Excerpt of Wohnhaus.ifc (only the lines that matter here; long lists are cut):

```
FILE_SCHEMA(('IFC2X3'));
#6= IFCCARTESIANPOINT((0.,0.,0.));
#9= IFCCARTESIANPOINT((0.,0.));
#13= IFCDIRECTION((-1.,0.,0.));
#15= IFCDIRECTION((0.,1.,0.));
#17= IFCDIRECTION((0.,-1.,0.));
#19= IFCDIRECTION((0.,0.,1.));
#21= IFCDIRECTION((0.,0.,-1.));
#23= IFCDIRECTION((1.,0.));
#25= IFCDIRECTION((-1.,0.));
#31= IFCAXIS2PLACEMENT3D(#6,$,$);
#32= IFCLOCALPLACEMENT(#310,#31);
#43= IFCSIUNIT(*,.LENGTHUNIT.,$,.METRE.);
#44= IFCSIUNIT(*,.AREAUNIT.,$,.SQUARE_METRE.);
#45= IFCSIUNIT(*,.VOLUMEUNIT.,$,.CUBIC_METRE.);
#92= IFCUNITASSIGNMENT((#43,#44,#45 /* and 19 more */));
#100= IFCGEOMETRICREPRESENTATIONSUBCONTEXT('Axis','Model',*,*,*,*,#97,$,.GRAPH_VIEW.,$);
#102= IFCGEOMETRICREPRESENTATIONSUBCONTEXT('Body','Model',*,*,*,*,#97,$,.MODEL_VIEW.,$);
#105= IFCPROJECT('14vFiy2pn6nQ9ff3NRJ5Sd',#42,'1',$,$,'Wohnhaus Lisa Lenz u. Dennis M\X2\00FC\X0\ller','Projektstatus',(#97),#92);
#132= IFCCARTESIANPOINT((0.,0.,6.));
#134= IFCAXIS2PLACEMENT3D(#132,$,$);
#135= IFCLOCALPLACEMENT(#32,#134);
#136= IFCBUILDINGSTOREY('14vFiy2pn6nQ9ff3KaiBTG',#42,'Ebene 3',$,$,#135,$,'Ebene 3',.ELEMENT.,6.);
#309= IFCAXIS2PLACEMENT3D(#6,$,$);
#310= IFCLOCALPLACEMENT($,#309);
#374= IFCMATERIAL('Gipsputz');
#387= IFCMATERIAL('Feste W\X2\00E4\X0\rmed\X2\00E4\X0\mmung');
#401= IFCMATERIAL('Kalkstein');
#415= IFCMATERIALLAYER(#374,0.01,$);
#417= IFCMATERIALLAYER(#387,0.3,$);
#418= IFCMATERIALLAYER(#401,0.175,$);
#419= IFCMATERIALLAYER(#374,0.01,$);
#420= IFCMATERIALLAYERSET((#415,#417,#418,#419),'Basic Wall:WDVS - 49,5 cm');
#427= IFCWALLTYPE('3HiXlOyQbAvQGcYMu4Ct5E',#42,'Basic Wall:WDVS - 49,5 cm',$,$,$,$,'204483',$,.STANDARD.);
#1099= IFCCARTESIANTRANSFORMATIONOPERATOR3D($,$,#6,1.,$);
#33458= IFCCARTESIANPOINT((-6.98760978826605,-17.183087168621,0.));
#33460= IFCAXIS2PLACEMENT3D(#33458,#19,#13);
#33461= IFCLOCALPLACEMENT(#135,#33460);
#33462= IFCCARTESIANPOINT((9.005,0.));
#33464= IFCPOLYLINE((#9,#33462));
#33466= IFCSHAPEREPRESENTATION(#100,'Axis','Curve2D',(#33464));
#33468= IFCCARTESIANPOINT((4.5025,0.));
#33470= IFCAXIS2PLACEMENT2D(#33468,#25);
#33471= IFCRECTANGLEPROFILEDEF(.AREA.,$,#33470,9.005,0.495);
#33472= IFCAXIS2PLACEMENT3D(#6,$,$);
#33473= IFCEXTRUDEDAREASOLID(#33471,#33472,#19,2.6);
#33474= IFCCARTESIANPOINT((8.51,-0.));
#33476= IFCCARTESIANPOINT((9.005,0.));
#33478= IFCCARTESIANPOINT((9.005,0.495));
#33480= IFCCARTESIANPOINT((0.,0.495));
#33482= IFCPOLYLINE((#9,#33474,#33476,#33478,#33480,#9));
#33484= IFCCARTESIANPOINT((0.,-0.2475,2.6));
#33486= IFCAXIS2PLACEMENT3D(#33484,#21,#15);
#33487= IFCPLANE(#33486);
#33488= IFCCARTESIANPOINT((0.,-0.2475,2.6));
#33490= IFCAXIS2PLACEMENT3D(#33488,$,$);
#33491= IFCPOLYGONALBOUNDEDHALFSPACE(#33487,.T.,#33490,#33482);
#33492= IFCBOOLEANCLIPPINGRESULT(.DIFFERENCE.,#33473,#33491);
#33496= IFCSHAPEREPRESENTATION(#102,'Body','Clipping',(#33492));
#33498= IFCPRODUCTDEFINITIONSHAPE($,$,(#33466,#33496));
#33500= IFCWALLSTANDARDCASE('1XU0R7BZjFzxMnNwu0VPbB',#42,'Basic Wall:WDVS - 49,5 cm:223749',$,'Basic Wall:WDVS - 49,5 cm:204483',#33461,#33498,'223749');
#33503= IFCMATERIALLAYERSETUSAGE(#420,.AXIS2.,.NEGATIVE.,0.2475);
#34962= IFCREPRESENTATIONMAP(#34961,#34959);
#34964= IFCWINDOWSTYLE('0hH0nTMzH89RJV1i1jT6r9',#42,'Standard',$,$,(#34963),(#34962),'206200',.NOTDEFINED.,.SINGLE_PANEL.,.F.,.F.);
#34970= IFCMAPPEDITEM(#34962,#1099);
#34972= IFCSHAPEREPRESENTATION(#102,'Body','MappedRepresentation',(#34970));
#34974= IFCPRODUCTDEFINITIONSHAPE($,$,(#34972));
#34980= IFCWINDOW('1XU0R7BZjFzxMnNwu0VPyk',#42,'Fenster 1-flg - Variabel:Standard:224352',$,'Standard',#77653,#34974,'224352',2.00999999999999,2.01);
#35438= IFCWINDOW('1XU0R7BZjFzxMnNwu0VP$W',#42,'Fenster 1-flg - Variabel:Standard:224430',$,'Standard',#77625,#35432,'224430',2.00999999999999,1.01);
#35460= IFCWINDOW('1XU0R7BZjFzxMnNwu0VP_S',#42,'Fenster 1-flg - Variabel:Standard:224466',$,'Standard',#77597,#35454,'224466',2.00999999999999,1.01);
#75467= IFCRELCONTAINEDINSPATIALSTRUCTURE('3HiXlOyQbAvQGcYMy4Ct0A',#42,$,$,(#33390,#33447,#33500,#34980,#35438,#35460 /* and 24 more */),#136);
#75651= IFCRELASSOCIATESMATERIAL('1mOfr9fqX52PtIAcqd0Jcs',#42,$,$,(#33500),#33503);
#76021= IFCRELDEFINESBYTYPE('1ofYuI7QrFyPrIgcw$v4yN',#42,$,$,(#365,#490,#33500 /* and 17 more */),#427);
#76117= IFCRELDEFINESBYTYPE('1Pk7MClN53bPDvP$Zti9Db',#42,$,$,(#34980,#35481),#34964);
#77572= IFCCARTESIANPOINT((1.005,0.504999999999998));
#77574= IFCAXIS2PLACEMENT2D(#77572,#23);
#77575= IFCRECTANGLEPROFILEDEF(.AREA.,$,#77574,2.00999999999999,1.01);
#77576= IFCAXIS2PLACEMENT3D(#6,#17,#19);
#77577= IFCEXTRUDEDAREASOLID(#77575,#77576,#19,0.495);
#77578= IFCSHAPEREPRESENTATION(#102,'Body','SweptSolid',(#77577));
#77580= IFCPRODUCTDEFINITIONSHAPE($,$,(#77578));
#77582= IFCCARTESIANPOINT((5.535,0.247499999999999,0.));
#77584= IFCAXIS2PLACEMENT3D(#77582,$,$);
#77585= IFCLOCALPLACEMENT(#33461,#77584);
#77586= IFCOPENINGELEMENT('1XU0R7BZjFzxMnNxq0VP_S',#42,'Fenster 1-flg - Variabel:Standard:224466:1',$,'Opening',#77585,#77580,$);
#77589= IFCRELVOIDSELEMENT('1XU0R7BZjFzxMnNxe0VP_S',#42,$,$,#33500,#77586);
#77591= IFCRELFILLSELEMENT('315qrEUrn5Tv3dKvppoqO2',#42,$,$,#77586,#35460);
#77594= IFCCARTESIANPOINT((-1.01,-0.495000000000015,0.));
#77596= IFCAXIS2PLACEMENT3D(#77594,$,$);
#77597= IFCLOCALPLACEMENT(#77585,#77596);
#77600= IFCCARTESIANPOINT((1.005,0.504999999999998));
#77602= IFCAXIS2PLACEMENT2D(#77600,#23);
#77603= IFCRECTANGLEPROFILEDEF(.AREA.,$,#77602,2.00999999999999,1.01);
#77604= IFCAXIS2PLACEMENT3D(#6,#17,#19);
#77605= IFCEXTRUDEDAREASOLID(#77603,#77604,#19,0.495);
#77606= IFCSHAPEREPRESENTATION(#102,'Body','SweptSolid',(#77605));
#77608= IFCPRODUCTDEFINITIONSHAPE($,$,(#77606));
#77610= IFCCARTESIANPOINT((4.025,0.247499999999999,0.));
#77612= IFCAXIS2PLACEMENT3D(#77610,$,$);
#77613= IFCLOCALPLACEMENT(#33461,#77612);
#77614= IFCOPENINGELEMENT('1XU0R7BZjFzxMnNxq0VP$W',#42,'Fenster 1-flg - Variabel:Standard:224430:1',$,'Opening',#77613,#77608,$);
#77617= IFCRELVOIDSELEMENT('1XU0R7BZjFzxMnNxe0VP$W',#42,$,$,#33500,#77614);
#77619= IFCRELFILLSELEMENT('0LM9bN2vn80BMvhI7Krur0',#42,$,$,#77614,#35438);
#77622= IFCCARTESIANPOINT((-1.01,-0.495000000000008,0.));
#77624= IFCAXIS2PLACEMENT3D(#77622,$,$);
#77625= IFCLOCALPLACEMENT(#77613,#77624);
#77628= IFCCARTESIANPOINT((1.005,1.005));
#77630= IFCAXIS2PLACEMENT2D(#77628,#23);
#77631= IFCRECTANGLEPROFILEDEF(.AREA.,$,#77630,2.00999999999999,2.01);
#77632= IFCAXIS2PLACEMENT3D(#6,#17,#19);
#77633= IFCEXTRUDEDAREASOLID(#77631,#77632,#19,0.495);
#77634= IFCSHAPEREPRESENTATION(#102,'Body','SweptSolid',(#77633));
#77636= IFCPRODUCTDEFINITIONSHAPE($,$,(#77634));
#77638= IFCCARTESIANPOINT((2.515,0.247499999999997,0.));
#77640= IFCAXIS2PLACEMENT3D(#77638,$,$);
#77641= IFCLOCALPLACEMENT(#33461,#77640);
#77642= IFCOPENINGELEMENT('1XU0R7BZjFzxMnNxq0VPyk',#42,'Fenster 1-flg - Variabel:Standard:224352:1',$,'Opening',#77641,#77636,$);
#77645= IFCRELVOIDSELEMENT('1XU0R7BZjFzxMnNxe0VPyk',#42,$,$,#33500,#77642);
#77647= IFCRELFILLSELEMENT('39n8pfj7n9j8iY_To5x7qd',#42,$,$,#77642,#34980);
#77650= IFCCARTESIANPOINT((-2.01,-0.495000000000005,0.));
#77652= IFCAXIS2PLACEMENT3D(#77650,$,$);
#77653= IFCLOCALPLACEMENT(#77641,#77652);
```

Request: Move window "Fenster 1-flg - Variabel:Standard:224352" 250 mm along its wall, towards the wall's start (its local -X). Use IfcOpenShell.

```python
import ifcopenshell
import ifcopenshell.api.geometry
import ifcopenshell.util.placement
import ifcopenshell.util.unit

model = ifcopenshell.open("Wohnhaus.ifc")
unit_scale = ifcopenshell.util.unit.calculate_unit_scale(model)

window = model.by_guid("1XU0R7BZjFzxMnNwu0VPyk")
opening = window.FillsVoids[0].RelatingOpeningElement
wall = opening.VoidsElements[0].RelatingBuildingElement

wall_matrix = ifcopenshell.util.placement.get_local_placement(wall.ObjectPlacement)
shift = wall_matrix[:3, 0] * -0.25 / unit_scale
before = ifcopenshell.util.placement.get_local_placement(window.ObjectPlacement)[:3, 3].copy()

# The window is placed relative to its opening, so it follows when the opening moves.
matrix = ifcopenshell.util.placement.get_local_placement(opening.ObjectPlacement)
matrix[:3, 3] += shift
ifcopenshell.api.geometry.edit_object_placement(
    model, product=opening, matrix=matrix, is_si=False, should_transform_children=True
)

after = ifcopenshell.util.placement.get_local_placement(window.ObjectPlacement)[:3, 3]
print("window moved by", (after - before).round(3) + 0.0)

model.write("Wohnhaus_edited.ifc")
```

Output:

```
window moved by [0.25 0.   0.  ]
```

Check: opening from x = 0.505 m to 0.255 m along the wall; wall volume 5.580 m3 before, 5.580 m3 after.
